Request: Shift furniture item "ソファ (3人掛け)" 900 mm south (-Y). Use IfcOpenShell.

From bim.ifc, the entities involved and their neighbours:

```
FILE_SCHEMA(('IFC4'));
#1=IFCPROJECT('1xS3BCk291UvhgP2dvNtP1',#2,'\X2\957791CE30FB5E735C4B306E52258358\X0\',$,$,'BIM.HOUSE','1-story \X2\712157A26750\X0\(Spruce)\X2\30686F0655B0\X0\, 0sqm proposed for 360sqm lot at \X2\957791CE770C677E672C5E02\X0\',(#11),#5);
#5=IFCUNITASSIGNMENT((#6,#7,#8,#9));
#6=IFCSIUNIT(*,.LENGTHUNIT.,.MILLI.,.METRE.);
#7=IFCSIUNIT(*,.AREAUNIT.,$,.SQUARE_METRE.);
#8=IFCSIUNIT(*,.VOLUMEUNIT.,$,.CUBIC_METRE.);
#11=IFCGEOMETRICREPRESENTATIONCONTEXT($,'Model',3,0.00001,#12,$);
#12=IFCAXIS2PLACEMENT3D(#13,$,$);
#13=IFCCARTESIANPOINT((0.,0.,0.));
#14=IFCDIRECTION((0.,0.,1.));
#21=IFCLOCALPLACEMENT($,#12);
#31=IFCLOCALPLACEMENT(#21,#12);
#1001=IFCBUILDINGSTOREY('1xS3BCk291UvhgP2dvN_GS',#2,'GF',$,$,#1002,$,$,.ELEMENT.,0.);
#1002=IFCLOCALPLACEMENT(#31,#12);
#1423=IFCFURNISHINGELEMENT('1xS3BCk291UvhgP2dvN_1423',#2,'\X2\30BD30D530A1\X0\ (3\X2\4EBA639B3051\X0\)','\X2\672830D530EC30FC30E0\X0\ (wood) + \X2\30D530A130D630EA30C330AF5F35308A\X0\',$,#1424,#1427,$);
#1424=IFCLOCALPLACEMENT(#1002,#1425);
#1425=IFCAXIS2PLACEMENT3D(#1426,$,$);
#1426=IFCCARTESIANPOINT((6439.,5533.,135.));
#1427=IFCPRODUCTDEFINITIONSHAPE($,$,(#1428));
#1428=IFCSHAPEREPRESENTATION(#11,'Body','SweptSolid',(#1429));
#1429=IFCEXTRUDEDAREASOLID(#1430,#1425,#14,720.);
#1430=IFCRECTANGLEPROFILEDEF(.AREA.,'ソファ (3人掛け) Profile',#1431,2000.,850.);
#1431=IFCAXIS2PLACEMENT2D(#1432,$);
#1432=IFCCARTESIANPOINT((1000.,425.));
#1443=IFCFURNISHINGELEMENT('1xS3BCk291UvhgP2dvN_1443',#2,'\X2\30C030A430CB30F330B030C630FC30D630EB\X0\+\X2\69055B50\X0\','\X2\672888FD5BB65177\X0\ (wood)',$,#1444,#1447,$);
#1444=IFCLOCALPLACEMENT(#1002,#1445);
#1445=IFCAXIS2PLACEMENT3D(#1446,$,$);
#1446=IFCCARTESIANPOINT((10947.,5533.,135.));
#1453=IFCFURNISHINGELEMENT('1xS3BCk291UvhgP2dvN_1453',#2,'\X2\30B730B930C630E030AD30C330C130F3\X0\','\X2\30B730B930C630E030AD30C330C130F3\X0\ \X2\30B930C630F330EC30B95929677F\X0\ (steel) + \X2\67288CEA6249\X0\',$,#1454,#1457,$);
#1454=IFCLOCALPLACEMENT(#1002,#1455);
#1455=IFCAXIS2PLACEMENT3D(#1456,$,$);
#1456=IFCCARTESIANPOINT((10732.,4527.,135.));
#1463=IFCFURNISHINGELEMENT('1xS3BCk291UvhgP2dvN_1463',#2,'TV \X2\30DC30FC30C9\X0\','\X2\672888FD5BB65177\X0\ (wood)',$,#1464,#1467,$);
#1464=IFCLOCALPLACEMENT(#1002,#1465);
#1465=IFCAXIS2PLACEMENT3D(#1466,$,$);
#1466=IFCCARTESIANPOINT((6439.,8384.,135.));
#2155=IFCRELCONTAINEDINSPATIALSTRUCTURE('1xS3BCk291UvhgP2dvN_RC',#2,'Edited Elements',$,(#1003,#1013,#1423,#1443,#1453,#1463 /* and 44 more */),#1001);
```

```python
import ifcopenshell
import ifcopenshell.api.geometry
import ifcopenshell.util.placement
import ifcopenshell.util.unit

model = ifcopenshell.open("bim.ifc")
unit_scale = ifcopenshell.util.unit.calculate_unit_scale(model)

item = model.by_guid("1xS3BCk291UvhgP2dvN_1423")
matrix = ifcopenshell.util.placement.get_local_placement(item.ObjectPlacement)
matrix[1, 3] -= 0.9 / unit_scale
ifcopenshell.api.geometry.edit_object_placement(model, product=item, matrix=matrix, is_si=False)

print(ifcopenshell.util.placement.get_local_placement(item.ObjectPlacement).round(3) + 0.0)

model.write("bim_updated.ifc")
```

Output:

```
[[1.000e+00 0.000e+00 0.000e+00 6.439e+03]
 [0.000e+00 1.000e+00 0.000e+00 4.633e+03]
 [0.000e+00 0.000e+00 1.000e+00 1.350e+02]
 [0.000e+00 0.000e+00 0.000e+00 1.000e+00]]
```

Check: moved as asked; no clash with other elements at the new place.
